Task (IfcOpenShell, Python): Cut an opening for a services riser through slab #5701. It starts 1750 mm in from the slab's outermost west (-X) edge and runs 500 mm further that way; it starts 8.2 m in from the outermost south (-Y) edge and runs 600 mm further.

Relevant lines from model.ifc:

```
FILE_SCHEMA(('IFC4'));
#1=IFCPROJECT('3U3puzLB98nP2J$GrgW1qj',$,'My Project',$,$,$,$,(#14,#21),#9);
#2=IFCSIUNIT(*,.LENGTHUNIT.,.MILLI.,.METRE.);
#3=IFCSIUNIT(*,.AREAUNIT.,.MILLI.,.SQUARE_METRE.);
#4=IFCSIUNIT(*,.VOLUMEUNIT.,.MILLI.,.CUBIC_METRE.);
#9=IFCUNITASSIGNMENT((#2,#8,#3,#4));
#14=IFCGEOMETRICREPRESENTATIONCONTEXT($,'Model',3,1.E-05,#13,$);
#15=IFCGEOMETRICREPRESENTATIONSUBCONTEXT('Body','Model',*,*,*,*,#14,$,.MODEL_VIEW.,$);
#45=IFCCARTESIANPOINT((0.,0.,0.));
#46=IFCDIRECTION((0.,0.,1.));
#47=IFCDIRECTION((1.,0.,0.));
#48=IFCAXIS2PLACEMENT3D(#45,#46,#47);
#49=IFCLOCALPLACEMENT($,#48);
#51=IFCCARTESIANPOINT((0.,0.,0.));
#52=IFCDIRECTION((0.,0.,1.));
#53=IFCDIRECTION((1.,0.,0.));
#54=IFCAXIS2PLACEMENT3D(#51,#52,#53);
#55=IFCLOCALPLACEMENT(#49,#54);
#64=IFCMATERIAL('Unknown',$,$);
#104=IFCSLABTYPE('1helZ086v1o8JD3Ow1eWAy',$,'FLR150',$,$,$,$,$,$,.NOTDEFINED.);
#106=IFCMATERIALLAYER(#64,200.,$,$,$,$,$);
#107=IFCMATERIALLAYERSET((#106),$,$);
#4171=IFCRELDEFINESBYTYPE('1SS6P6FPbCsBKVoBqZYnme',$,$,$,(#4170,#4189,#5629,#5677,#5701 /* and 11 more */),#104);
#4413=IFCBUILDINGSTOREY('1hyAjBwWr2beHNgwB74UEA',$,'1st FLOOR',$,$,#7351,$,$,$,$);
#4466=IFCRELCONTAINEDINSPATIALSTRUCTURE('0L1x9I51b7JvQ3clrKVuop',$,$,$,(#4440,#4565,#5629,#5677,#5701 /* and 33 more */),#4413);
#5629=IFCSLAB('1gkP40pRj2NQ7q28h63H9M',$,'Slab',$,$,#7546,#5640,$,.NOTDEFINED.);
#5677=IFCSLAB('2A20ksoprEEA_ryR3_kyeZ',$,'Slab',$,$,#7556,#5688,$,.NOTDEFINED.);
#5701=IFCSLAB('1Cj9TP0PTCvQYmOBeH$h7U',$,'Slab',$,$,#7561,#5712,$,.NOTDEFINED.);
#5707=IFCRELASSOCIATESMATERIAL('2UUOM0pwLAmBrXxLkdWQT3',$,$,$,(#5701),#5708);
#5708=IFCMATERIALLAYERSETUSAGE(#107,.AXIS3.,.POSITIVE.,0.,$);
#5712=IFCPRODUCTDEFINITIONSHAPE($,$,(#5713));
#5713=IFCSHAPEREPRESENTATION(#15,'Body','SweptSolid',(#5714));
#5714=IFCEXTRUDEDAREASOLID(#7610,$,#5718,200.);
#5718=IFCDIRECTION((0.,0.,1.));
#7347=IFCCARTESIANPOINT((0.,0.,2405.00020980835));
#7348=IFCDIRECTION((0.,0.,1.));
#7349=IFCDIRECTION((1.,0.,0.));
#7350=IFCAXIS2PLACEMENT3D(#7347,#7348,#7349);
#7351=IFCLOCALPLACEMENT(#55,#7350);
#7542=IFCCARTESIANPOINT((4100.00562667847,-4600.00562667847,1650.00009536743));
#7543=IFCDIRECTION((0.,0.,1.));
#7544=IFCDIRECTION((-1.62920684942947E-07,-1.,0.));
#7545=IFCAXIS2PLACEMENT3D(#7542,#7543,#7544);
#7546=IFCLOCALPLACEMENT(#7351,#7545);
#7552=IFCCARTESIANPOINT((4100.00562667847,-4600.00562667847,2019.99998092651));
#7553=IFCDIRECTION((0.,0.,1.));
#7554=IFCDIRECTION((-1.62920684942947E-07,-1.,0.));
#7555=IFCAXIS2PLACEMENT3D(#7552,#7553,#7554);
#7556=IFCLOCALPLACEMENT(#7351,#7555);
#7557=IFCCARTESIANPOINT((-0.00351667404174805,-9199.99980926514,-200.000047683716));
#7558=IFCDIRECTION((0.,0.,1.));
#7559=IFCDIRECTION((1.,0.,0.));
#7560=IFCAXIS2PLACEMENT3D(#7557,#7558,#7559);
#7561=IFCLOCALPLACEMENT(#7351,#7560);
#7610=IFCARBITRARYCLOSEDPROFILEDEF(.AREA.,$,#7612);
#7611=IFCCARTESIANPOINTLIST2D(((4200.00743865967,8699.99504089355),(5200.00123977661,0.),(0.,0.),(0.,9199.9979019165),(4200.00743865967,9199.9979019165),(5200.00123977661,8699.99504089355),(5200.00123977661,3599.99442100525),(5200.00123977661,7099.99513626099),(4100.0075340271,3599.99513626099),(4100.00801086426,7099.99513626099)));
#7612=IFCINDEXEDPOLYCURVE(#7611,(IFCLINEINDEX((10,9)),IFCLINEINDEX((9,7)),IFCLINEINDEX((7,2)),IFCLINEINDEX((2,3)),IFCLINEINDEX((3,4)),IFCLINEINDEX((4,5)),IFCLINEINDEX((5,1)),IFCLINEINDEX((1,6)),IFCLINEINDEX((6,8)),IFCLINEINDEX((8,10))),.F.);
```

```python
import numpy as np
import ifcopenshell
import ifcopenshell.api.feature
import ifcopenshell.api.geometry
import ifcopenshell.api.root
import ifcopenshell.geom
import ifcopenshell.util.placement
import ifcopenshell.util.representation
import ifcopenshell.util.shape
import ifcopenshell.util.unit

model = ifcopenshell.open("model.ifc")
unit_scale = ifcopenshell.util.unit.calculate_unit_scale(model)
settings = ifcopenshell.geom.settings()


def volume(element):
    """Net volume in cubic metres, openings subtracted."""
    shape = ifcopenshell.geom.create_shape(settings, element)
    return ifcopenshell.util.shape.get_volume(shape.geometry)


slab = model.by_id(5701)
before = volume(slab)

# Extent in the slab's own axes, in metres. The edges named are its -X and -Y sides.
slab_shape = ifcopenshell.geom.create_shape(settings, slab)
vertices = ifcopenshell.util.shape.get_vertices(slab_shape.geometry)
x_min, y_min, bottom = vertices.min(axis=0)
top = vertices[:, 2].max()

opening = ifcopenshell.api.root.create_entity(model, ifc_class="IfcOpeningElement", name="Services riser opening", predefined_type="OPENING")
context = ifcopenshell.util.representation.get_context(model, "Model", "Body", "MODEL_VIEW")
width, depth = 0.5, 0.6
outline = [(0.0, 0.0), (width, 0.0), (width, depth), (0.0, depth), (0.0, 0.0)]
# Overshoot both faces by 50 mm so the cut is clean.
shape = ifcopenshell.api.geometry.add_slab_representation(
    model, context=context, depth=top - bottom + 0.1, polyline=outline
)
ifcopenshell.api.geometry.assign_representation(model, product=opening, representation=shape)

matrix = ifcopenshell.util.placement.get_local_placement(slab.ObjectPlacement)
matrix[:, 3] = matrix @ np.append(np.array([x_min + 1.75, y_min + 8.2, bottom - 0.05]) / unit_scale, 1.0)
ifcopenshell.api.geometry.edit_object_placement(model, product=opening, matrix=matrix, is_si=False)
ifcopenshell.api.feature.add_feature(model, feature=opening, element=slab)

after = volume(slab)

print(f"slab volume {before:.3f} -> {after:.3f} m3")

model.write("model_updated.ifc")
```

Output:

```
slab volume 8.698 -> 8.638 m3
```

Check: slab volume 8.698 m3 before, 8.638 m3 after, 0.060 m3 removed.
